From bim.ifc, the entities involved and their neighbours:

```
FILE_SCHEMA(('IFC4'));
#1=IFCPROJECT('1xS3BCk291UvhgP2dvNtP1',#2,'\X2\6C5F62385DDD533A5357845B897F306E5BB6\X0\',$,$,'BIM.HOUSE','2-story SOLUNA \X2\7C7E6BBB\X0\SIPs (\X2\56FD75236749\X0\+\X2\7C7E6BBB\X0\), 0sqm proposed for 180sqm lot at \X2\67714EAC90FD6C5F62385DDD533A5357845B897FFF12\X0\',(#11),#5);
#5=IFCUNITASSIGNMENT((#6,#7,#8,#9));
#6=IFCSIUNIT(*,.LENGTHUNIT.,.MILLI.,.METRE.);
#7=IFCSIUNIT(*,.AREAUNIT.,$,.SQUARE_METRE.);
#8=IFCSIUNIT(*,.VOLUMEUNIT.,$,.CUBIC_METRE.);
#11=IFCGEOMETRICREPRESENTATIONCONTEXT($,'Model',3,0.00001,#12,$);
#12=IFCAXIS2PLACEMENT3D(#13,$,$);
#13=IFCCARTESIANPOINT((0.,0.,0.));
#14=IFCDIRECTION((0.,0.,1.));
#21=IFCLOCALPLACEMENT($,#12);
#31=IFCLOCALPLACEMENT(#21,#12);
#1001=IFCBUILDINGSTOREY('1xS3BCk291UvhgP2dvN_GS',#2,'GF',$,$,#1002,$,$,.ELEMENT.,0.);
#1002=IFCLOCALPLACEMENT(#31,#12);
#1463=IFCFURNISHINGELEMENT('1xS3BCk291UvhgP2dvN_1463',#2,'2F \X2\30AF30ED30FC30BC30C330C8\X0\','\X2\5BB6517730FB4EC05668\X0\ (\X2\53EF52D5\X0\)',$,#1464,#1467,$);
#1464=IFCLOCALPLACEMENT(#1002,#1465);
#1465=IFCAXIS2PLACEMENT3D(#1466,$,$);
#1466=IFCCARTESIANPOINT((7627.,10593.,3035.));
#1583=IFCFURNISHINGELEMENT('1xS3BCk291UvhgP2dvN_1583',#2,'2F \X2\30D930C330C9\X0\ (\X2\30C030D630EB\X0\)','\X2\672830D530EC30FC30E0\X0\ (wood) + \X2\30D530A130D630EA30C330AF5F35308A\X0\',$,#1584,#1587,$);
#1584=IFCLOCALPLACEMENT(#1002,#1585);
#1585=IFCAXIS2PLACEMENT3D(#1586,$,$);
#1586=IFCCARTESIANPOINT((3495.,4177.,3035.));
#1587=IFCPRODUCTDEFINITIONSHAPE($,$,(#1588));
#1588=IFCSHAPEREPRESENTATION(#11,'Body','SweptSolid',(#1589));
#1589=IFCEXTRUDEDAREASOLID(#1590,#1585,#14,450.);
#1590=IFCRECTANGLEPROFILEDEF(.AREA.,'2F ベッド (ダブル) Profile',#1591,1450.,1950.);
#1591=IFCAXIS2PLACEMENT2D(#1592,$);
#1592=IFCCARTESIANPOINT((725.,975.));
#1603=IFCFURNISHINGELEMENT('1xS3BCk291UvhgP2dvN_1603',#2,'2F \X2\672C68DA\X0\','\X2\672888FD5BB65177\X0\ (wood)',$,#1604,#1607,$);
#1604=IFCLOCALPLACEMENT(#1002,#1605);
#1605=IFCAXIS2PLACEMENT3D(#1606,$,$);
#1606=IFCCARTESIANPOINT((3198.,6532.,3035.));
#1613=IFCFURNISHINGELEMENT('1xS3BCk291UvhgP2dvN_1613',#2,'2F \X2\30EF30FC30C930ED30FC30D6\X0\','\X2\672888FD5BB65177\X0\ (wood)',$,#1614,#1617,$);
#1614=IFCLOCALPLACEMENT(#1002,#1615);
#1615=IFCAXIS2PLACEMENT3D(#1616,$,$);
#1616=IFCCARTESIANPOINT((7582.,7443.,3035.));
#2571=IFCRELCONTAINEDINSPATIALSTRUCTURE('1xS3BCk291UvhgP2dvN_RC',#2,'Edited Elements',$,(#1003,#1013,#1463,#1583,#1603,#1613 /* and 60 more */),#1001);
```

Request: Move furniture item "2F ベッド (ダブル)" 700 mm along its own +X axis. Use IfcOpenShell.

```python
import ifcopenshell
import ifcopenshell.api.geometry
import ifcopenshell.util.placement
import ifcopenshell.util.unit

model = ifcopenshell.open("bim.ifc")
unit_scale = ifcopenshell.util.unit.calculate_unit_scale(model)

item = model.by_guid("1xS3BCk291UvhgP2dvN_1583")
matrix = ifcopenshell.util.placement.get_local_placement(item.ObjectPlacement)
matrix[:3, 3] += matrix[:3, 0] * 0.7 / unit_scale
ifcopenshell.api.geometry.edit_object_placement(model, product=item, matrix=matrix, is_si=False)

print(ifcopenshell.util.placement.get_local_placement(item.ObjectPlacement).round(3) + 0.0)

model.write("bim_rev.ifc")
```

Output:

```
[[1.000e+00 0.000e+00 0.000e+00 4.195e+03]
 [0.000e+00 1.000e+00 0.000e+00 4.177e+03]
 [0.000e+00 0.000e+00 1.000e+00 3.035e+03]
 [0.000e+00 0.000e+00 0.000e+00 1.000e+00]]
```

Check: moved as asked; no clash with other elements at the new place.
